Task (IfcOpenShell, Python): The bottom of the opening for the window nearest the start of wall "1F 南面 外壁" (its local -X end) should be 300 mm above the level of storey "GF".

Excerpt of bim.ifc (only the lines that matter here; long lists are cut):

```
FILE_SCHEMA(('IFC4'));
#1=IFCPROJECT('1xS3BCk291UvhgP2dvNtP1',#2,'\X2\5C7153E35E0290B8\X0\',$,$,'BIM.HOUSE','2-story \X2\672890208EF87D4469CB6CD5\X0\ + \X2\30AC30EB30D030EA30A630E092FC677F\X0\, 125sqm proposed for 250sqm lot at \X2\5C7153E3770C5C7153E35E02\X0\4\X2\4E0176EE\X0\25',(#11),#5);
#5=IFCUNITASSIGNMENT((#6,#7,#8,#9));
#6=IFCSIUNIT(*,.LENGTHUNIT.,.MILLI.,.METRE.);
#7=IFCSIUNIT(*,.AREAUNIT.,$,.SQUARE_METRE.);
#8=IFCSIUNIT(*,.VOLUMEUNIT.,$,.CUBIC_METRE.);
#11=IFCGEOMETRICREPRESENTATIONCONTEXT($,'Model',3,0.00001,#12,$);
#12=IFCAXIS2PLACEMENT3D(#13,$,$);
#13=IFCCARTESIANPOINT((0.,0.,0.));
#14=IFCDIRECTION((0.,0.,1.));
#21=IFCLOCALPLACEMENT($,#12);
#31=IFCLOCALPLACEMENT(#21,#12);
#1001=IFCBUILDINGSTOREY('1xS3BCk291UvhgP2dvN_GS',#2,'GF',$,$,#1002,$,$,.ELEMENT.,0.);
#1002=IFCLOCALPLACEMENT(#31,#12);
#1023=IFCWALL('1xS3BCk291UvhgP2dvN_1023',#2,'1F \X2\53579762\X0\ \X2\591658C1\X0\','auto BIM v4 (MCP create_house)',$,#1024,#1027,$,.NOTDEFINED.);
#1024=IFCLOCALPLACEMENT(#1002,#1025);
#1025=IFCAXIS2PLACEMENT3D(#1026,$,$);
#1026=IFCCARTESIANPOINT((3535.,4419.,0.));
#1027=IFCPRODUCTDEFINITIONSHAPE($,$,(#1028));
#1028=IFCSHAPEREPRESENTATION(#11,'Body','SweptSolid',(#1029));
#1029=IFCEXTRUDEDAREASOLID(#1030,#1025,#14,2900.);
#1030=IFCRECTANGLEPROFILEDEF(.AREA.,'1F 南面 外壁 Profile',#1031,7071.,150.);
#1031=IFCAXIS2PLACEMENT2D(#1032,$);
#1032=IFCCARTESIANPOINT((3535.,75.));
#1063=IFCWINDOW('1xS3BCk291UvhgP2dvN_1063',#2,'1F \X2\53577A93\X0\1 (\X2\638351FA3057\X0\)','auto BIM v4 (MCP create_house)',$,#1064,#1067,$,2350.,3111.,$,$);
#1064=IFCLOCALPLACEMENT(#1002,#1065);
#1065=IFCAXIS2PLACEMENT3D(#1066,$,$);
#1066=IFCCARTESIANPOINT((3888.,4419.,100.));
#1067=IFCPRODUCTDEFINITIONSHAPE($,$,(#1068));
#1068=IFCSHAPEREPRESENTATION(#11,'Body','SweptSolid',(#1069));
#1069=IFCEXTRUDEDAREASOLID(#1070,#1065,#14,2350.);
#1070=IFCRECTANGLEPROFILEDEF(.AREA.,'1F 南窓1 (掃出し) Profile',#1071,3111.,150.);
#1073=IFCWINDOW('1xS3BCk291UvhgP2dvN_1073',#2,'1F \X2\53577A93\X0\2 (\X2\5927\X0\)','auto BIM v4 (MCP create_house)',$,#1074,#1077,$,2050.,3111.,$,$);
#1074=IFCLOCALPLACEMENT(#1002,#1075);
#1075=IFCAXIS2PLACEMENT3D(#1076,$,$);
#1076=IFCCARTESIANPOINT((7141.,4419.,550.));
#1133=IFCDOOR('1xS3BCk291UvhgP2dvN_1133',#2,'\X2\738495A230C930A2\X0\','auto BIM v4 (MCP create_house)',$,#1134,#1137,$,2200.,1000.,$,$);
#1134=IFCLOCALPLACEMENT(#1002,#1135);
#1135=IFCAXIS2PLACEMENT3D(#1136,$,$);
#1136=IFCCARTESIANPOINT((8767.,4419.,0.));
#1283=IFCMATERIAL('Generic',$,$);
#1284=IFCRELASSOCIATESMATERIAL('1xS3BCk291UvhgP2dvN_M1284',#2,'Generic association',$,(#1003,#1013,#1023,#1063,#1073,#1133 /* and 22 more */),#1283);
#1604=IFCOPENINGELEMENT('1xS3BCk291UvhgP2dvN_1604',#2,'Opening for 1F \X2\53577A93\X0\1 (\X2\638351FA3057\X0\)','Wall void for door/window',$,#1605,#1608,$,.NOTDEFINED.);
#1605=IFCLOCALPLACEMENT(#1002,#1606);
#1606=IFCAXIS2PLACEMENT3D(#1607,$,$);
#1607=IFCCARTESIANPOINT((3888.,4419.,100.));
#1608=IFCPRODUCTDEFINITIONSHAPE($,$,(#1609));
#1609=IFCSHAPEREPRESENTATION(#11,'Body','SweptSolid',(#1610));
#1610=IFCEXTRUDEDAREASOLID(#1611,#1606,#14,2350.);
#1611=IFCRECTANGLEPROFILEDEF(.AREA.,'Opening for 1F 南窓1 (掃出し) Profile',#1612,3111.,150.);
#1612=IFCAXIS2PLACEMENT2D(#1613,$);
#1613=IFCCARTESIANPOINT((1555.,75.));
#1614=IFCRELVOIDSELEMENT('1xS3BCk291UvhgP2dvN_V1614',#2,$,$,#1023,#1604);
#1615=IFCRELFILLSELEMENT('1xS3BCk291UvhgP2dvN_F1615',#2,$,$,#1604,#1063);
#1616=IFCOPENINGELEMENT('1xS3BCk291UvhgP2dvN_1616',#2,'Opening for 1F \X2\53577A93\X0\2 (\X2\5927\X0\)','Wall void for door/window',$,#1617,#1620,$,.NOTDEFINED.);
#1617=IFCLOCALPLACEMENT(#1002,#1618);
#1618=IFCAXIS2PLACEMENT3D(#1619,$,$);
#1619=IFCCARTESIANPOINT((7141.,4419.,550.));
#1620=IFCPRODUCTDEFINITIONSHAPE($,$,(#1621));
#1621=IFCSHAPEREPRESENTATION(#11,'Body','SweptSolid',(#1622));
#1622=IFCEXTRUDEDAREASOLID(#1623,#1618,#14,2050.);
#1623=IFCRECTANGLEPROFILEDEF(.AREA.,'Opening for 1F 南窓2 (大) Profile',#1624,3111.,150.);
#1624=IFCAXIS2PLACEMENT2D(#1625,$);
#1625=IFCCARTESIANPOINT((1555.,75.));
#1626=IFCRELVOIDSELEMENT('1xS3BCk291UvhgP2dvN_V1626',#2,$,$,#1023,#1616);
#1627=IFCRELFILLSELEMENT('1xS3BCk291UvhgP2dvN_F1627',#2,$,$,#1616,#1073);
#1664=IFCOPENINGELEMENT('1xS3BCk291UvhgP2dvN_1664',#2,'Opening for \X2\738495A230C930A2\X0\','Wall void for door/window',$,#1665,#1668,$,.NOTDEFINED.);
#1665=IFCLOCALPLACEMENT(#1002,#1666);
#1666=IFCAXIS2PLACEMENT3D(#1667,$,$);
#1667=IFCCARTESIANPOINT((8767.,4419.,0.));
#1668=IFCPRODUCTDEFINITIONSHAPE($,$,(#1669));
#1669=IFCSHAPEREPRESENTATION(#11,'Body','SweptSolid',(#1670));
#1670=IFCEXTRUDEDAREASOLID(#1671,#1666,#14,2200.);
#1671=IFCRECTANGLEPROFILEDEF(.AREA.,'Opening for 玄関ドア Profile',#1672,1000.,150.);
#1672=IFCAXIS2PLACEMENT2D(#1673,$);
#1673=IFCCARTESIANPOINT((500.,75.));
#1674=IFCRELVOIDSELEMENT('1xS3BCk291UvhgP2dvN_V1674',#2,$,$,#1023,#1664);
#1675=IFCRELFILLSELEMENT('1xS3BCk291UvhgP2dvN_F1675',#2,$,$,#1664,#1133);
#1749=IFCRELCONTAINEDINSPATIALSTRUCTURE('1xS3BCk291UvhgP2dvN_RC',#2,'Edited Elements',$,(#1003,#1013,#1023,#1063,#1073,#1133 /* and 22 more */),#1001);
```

```python
import numpy as np
import ifcopenshell
import ifcopenshell.api.geometry
import ifcopenshell.geom
import ifcopenshell.util.element
import ifcopenshell.util.placement
import ifcopenshell.util.shape
import ifcopenshell.util.unit

model = ifcopenshell.open("bim.ifc")
unit_scale = ifcopenshell.util.unit.calculate_unit_scale(model)

window = model.by_guid("1xS3BCk291UvhgP2dvN_1063")
opening = window.FillsVoids[0].RelatingOpeningElement
storey = ifcopenshell.util.element.get_container(window, ifc_class="IfcBuildingStorey")
level = ifcopenshell.util.placement.get_local_placement(storey.ObjectPlacement)[2, 3]

# The opening's origin need not be at the sill, so measure its lowest point.
shape = ifcopenshell.geom.create_shape(ifcopenshell.geom.settings(), opening)
bottom = ifcopenshell.util.shape.get_shape_bottom_elevation(shape, shape.geometry) / unit_scale
dz = level + 0.3 / unit_scale - bottom

shift = np.array([0.0, 0.0, dz])
# The window is not placed relative to its opening, so move both.
for product in (opening, window):
    matrix = ifcopenshell.util.placement.get_local_placement(product.ObjectPlacement)
    matrix[:3, 3] += shift
    ifcopenshell.api.geometry.edit_object_placement(model, product=product, matrix=matrix, is_si=False)

print(f"moved by {dz * unit_scale:+.3f} m")

model.write("bim_updated.ifc")
```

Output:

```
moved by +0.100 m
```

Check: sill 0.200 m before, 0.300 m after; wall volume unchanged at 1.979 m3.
